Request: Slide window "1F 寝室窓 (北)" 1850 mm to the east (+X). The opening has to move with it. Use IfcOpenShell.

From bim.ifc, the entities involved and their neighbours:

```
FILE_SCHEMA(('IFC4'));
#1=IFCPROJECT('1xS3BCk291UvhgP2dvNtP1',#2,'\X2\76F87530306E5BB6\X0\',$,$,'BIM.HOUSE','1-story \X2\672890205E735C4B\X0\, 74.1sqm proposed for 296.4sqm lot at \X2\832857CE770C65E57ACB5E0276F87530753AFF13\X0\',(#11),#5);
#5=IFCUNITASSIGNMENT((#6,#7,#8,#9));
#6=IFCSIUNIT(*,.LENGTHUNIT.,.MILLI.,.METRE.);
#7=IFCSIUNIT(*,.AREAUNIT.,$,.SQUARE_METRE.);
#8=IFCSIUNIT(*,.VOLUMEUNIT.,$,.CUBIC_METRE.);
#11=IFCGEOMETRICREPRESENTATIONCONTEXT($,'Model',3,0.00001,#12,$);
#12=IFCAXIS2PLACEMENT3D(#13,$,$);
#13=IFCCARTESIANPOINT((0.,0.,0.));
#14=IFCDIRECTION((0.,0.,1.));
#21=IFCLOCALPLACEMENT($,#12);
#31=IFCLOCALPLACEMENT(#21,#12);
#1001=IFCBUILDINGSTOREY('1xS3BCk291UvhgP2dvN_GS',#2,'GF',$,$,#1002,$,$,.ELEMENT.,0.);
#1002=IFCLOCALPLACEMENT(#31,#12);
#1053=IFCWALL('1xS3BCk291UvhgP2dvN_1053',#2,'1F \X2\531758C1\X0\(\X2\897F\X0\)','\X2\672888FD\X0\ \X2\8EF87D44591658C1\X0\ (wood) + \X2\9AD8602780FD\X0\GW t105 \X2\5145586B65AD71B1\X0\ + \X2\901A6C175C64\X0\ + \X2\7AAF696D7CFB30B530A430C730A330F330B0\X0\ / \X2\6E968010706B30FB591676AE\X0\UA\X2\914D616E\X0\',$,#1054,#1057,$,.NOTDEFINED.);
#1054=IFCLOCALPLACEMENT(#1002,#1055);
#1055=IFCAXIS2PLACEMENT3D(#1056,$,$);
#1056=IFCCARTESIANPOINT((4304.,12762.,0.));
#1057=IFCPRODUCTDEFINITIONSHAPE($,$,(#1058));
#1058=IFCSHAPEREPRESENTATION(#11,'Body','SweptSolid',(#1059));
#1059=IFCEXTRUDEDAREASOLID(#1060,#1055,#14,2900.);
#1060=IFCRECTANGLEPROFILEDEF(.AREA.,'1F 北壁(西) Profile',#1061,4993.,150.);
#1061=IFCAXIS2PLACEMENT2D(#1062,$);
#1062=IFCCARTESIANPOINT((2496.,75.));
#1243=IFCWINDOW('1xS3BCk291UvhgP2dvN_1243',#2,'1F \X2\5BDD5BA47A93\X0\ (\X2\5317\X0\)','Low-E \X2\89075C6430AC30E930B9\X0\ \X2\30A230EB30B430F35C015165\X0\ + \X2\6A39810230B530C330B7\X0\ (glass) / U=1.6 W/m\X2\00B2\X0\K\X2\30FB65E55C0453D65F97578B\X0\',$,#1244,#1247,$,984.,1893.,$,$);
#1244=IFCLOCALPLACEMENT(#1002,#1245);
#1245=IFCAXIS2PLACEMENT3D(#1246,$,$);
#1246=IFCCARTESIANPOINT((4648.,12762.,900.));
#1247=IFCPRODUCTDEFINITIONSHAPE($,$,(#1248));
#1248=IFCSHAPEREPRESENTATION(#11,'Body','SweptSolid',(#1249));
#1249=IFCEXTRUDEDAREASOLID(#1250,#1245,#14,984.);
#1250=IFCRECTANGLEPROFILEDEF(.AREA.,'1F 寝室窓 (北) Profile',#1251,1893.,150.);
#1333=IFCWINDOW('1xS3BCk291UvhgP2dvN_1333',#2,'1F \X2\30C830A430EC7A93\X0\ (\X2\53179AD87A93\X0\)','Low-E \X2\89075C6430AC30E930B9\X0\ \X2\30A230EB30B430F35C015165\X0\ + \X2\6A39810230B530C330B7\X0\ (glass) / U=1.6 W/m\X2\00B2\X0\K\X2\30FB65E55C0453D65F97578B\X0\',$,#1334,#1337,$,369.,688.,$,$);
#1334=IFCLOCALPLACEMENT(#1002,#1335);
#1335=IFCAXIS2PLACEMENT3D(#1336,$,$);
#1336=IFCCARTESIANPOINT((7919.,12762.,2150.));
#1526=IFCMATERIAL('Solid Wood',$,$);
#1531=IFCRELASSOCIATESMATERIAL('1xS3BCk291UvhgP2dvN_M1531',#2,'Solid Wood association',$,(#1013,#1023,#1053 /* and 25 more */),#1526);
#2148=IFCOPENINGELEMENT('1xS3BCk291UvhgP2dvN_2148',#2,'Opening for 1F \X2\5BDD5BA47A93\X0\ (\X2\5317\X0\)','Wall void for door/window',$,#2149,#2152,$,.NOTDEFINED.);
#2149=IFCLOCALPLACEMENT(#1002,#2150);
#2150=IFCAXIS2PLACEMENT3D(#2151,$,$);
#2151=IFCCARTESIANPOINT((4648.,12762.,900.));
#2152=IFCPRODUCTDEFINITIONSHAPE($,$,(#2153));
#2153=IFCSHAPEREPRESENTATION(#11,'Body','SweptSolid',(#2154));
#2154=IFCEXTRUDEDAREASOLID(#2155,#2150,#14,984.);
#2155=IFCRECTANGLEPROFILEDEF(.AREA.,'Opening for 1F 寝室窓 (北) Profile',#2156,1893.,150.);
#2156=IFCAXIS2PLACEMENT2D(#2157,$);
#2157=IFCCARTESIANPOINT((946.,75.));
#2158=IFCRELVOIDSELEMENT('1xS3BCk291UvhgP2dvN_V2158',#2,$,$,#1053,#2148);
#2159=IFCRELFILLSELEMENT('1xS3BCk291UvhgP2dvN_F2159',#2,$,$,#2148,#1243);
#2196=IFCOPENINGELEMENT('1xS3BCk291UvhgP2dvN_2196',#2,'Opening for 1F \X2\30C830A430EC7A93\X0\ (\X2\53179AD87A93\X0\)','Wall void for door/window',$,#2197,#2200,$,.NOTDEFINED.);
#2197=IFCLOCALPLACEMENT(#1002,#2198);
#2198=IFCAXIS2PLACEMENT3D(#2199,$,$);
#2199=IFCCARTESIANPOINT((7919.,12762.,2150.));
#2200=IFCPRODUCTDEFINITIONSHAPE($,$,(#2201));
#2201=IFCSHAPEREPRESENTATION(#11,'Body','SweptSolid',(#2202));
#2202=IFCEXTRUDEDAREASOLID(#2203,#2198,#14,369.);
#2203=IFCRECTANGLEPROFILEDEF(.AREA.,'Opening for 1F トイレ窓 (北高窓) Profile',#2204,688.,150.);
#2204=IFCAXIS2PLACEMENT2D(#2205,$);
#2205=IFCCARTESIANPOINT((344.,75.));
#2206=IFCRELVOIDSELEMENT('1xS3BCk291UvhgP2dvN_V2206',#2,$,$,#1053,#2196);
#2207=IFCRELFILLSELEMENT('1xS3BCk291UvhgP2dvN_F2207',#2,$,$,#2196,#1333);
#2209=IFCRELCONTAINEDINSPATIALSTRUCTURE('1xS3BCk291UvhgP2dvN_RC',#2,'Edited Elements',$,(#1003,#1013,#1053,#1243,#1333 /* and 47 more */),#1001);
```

```python
import ifcopenshell
import ifcopenshell.api.geometry
import ifcopenshell.util.placement

model = ifcopenshell.open("bim.ifc")

window = model.by_guid("1xS3BCk291UvhgP2dvN_1243")
opening = window.FillsVoids[0].RelatingOpeningElement
wall = opening.VoidsElements[0].RelatingBuildingElement

wall_matrix = ifcopenshell.util.placement.get_local_placement(wall.ObjectPlacement)
shift = wall_matrix[:3, 0] * 1850.0
before = ifcopenshell.util.placement.get_local_placement(window.ObjectPlacement)[:3, 3].copy()

# The window is not placed relative to its opening, so move both.
for product in (opening, window):
    matrix = ifcopenshell.util.placement.get_local_placement(product.ObjectPlacement)
    matrix[:3, 3] += shift
    ifcopenshell.api.geometry.edit_object_placement(model, product=product, matrix=matrix, is_si=False)

after = ifcopenshell.util.placement.get_local_placement(window.ObjectPlacement)[:3, 3]
print("window moved by", (after - before).round(3) + 0.0)

model.write("bim_updated.ifc")
```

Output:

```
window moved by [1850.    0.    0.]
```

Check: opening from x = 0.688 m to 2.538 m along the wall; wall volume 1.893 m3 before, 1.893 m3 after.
